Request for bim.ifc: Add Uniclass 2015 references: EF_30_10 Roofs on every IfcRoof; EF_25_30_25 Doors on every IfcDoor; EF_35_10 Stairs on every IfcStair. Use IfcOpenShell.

First a look at what the model holds.

```python
import ifcopenshell

model = ifcopenshell.open("bim.ifc")
print(model.schema)
print("classifications:", [c.Name for c in model.by_type("IfcClassification")])
for ifc_class in ("IfcDoor", "IfcRoof", "IfcStair", "IfcWall", "IfcWindow"):
    print(ifc_class, len(model.by_type(ifc_class)))
```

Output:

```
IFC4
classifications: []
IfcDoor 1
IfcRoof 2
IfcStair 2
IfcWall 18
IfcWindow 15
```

```python
import ifcopenshell
import ifcopenshell.api.classification

model = ifcopenshell.open("bim.ifc")

system = ifcopenshell.api.classification.add_classification(model, classification="Uniclass 2015")

codes = {
    "IfcRoof": ("EF_30_10", "Roofs"),
    "IfcDoor": ("EF_25_30_25", "Doors"),
    "IfcStair": ("EF_35_10", "Stairs"),
}
for ifc_class, (code, name) in codes.items():
    products = model.by_type(ifc_class)
    ifcopenshell.api.classification.add_reference(
        model, products=products, classification=system, identification=code, name=name
    )
    print(code, len(products))

model.write("bim_updated.ifc")
```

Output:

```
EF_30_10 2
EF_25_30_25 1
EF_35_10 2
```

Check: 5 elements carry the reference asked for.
